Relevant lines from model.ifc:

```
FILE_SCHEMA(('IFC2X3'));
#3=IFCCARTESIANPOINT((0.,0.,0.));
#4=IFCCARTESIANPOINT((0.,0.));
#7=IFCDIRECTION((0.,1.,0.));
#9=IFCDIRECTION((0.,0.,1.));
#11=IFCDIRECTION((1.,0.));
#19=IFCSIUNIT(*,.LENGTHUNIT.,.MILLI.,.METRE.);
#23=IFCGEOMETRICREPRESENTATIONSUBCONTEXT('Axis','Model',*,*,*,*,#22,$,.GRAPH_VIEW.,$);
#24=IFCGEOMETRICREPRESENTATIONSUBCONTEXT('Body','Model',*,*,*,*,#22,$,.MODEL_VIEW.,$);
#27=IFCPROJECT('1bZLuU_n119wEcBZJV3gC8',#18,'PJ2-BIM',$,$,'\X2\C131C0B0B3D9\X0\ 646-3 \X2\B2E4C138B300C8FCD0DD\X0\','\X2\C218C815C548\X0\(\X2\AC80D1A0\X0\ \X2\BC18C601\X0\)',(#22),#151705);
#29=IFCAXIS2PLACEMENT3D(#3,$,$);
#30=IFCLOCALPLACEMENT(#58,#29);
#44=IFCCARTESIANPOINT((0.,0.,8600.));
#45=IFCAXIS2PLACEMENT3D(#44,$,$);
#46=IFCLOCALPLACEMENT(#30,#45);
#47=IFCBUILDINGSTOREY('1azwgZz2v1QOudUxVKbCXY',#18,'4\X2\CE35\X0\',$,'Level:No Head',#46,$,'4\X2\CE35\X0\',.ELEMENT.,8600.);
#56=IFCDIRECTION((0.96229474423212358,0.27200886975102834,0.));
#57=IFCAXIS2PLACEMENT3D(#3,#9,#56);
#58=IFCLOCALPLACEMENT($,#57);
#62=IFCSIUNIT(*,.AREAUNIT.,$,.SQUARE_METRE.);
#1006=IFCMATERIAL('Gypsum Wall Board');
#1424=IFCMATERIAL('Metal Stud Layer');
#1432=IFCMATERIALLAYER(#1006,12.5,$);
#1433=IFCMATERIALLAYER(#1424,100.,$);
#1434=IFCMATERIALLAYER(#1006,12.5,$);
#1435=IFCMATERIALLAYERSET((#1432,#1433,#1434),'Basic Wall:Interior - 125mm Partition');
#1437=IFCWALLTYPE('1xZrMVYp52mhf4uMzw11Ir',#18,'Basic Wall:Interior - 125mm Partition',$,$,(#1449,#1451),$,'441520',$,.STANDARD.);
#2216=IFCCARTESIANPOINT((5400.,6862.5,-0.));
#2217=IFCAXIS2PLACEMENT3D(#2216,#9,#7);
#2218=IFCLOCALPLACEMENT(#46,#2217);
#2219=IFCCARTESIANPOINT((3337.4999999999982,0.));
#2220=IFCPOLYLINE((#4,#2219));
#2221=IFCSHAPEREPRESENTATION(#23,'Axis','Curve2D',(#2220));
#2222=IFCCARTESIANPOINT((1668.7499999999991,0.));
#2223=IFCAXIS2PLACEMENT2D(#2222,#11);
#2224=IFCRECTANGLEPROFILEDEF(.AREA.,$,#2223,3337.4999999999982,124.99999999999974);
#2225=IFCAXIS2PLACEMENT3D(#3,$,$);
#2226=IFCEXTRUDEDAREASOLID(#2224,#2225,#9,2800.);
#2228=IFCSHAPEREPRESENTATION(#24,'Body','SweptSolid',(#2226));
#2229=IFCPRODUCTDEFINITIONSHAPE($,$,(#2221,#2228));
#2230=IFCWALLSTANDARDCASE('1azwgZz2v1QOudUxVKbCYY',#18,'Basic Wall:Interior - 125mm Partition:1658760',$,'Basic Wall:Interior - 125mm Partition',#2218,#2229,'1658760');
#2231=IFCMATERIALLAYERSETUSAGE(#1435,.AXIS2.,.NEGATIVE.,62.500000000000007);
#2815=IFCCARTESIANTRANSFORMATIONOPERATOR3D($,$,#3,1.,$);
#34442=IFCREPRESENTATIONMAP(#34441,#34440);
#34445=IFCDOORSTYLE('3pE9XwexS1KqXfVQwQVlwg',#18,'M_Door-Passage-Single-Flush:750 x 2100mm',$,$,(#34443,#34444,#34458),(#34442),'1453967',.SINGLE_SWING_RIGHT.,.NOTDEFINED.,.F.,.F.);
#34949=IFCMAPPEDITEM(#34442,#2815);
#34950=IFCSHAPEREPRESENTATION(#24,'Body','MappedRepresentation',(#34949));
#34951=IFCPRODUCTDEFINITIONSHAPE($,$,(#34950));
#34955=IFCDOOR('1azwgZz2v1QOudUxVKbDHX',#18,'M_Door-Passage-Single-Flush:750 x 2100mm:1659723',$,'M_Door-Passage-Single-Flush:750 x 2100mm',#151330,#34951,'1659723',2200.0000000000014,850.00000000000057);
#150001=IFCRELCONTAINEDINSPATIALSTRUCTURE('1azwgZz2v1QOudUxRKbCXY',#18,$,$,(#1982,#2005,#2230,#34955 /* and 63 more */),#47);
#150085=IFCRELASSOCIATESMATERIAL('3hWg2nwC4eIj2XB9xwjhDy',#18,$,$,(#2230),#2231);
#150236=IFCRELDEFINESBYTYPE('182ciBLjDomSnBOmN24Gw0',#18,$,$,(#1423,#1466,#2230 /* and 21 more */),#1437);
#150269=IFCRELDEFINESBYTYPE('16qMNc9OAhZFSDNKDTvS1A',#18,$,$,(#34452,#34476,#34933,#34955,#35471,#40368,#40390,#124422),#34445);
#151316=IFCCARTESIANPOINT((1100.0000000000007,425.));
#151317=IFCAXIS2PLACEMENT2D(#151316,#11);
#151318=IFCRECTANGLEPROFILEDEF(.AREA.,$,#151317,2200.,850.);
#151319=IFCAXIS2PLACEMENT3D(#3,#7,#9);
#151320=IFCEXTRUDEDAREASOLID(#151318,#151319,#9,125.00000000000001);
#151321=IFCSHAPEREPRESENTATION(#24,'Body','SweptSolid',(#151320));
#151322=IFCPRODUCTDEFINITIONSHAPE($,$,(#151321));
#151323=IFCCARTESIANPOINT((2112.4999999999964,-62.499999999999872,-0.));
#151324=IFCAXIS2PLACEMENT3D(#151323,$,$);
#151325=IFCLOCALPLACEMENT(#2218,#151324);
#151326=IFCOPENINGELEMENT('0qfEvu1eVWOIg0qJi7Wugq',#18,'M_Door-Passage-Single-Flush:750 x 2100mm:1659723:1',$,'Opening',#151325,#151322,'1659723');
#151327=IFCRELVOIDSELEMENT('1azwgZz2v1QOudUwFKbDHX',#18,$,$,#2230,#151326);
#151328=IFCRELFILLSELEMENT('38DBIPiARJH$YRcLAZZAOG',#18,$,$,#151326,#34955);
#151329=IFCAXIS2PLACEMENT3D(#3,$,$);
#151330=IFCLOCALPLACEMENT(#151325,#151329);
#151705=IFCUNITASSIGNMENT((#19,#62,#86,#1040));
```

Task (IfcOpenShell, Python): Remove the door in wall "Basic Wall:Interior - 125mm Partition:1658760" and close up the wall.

```python
import ifcopenshell
import ifcopenshell.api.feature
import ifcopenshell.api.root
import ifcopenshell.geom
import ifcopenshell.util.shape

model = ifcopenshell.open("model.ifc")
settings = ifcopenshell.geom.settings()


def volume(element):
    """Net volume in cubic metres, openings subtracted."""
    shape = ifcopenshell.geom.create_shape(settings, element)
    return ifcopenshell.util.shape.get_volume(shape.geometry)


door = model.by_guid("1azwgZz2v1QOudUxVKbDHX")
opening = door.FillsVoids[0].RelatingOpeningElement
wall = opening.VoidsElements[0].RelatingBuildingElement
before = volume(wall)

ifcopenshell.api.root.remove_product(model, product=door)
ifcopenshell.api.feature.remove_feature(model, feature=opening)

after = volume(wall)

print(f"wall volume {before:.3f} -> {after:.3f} m3")

model.write("model-out.ifc")
```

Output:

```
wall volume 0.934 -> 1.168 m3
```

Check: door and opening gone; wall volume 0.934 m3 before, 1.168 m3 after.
